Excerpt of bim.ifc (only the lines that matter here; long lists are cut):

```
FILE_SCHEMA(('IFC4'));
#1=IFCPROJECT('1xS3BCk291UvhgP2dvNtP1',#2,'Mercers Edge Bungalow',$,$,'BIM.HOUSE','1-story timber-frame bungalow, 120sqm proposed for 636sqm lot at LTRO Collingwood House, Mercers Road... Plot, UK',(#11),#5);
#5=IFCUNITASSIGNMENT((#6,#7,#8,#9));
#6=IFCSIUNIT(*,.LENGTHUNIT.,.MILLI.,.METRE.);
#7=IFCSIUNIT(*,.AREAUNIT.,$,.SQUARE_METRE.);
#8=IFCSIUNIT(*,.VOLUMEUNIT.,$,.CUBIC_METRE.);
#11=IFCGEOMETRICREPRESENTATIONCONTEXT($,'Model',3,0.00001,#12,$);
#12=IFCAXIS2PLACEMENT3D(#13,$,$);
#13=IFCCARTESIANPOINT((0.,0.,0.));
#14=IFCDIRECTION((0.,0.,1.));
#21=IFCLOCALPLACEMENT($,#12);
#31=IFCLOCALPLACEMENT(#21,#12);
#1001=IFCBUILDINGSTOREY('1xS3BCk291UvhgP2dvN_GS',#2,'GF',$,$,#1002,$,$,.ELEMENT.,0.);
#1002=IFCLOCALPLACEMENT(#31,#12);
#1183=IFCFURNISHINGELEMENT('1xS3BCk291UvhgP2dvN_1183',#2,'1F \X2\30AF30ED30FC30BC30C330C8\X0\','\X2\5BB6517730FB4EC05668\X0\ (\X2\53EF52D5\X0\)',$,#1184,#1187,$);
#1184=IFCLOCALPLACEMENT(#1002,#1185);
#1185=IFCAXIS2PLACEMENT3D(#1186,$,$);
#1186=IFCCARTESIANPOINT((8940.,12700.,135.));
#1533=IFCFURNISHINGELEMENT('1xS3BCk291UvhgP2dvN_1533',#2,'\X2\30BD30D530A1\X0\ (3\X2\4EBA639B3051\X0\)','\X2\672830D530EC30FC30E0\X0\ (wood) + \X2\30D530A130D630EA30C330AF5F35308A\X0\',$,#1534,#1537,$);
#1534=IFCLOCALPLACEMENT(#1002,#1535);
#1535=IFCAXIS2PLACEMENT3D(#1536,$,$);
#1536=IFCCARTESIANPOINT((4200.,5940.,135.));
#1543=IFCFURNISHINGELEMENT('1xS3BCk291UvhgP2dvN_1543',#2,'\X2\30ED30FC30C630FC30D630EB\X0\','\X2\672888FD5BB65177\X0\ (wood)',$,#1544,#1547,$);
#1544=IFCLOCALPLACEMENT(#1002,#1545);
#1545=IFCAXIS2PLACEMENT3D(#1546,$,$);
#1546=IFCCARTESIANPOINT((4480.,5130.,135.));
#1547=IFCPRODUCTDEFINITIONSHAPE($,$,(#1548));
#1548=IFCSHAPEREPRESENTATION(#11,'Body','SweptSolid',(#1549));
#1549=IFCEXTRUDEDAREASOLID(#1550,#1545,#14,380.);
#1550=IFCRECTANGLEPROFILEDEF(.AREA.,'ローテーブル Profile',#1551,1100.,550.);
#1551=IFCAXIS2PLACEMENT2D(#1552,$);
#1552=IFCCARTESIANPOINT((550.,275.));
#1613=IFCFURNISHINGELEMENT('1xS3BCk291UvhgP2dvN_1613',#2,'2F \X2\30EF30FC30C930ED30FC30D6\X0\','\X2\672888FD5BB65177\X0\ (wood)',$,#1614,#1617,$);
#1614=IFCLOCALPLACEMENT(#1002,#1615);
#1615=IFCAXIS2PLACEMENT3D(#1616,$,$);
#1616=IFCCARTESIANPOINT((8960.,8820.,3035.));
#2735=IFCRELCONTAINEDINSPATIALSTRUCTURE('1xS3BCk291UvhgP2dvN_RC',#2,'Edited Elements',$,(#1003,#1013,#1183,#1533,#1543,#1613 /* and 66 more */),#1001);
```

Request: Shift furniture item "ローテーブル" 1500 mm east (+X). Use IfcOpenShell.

```python
import ifcopenshell
import ifcopenshell.api.geometry
import ifcopenshell.util.placement
import ifcopenshell.util.unit

model = ifcopenshell.open("bim.ifc")
unit_scale = ifcopenshell.util.unit.calculate_unit_scale(model)

item = model.by_guid("1xS3BCk291UvhgP2dvN_1543")
matrix = ifcopenshell.util.placement.get_local_placement(item.ObjectPlacement)
matrix[0, 3] += 1.5 / unit_scale
ifcopenshell.api.geometry.edit_object_placement(model, product=item, matrix=matrix, is_si=False)

print(ifcopenshell.util.placement.get_local_placement(item.ObjectPlacement).round(3) + 0.0)

model.write("bim_edited.ifc")
```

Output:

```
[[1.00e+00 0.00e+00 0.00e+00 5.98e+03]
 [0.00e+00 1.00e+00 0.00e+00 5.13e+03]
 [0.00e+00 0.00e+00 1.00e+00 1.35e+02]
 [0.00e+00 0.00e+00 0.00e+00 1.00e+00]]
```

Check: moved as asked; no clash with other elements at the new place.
